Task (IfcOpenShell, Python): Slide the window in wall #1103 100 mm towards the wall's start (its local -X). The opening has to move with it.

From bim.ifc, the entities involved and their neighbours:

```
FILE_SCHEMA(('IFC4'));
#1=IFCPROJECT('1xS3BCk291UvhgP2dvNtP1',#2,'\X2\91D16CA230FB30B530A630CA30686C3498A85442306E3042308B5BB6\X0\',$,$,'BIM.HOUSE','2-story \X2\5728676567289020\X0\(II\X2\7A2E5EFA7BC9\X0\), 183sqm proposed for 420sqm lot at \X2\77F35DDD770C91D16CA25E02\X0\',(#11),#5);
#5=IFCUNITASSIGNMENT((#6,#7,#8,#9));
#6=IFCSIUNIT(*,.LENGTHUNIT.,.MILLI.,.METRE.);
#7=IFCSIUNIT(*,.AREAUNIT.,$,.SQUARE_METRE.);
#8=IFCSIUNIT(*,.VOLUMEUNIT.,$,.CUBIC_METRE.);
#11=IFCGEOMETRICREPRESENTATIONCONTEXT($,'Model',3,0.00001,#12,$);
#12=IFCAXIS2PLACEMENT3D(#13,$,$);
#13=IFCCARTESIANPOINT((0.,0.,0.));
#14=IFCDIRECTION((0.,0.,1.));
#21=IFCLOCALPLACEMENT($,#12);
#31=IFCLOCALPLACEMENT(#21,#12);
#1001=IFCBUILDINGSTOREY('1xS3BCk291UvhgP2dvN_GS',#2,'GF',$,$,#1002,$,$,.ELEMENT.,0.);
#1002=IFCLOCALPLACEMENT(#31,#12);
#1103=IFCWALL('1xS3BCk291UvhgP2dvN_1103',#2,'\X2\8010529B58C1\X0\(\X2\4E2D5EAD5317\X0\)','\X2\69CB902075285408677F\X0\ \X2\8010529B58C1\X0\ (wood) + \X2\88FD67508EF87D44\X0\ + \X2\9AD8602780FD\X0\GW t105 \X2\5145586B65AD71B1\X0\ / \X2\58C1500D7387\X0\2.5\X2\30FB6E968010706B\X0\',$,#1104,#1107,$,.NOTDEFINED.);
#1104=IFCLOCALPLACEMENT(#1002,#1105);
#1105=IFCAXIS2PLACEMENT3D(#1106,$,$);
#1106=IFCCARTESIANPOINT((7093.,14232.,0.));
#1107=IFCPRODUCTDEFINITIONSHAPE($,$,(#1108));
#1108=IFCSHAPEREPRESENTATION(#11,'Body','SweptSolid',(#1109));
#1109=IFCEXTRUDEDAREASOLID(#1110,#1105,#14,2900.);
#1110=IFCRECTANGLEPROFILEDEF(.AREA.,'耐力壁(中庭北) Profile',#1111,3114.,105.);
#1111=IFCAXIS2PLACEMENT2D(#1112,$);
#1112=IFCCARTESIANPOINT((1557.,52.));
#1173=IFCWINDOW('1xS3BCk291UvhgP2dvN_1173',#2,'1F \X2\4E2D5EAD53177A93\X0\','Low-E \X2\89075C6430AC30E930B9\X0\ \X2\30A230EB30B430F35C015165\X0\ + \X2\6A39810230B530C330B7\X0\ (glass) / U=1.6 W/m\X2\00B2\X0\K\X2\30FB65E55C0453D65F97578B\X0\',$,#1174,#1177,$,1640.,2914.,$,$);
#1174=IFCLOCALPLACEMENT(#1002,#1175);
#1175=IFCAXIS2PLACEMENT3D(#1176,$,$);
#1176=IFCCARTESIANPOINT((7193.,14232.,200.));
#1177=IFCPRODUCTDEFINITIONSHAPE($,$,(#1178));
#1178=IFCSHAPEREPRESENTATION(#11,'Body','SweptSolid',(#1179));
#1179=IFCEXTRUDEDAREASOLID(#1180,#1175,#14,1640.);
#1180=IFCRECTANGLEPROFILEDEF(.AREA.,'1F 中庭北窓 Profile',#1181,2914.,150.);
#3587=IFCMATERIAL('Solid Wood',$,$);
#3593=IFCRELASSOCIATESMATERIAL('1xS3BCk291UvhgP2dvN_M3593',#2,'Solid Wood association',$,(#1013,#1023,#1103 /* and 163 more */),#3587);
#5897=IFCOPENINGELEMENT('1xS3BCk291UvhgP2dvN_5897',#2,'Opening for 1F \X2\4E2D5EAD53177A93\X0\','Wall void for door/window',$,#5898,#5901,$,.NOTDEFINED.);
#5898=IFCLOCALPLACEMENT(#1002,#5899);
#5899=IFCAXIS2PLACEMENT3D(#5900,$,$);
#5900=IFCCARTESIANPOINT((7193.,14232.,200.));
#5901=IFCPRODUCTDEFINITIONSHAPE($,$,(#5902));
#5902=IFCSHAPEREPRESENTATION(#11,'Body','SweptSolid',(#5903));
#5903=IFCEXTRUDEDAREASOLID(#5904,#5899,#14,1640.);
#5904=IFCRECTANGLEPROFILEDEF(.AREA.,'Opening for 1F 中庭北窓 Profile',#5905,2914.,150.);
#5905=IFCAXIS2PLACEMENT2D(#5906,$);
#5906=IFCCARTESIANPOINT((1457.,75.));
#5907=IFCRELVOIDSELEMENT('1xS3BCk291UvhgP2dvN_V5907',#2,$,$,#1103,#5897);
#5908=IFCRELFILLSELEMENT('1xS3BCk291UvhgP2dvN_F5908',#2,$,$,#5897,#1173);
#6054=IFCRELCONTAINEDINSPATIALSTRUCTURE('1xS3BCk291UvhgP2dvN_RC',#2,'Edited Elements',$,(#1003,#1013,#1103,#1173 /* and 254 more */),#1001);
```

```python
import ifcopenshell
import ifcopenshell.api.geometry
import ifcopenshell.util.placement
import ifcopenshell.util.unit

model = ifcopenshell.open("bim.ifc")
unit_scale = ifcopenshell.util.unit.calculate_unit_scale(model)

window = model.by_guid("1xS3BCk291UvhgP2dvN_1173")
opening = window.FillsVoids[0].RelatingOpeningElement
wall = opening.VoidsElements[0].RelatingBuildingElement

wall_matrix = ifcopenshell.util.placement.get_local_placement(wall.ObjectPlacement)
shift = wall_matrix[:3, 0] * -0.1 / unit_scale
before = ifcopenshell.util.placement.get_local_placement(window.ObjectPlacement)[:3, 3].copy()

# The window is not placed relative to its opening, so move both.
for product in (opening, window):
    matrix = ifcopenshell.util.placement.get_local_placement(product.ObjectPlacement)
    matrix[:3, 3] += shift
    ifcopenshell.api.geometry.edit_object_placement(model, product=product, matrix=matrix, is_si=False)

after = ifcopenshell.util.placement.get_local_placement(window.ObjectPlacement)[:3, 3]
print("window moved by", (after - before).round(3) + 0.0)

model.write("bim_updated.ifc")
```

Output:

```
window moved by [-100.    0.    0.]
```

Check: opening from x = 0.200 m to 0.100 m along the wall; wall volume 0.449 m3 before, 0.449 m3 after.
